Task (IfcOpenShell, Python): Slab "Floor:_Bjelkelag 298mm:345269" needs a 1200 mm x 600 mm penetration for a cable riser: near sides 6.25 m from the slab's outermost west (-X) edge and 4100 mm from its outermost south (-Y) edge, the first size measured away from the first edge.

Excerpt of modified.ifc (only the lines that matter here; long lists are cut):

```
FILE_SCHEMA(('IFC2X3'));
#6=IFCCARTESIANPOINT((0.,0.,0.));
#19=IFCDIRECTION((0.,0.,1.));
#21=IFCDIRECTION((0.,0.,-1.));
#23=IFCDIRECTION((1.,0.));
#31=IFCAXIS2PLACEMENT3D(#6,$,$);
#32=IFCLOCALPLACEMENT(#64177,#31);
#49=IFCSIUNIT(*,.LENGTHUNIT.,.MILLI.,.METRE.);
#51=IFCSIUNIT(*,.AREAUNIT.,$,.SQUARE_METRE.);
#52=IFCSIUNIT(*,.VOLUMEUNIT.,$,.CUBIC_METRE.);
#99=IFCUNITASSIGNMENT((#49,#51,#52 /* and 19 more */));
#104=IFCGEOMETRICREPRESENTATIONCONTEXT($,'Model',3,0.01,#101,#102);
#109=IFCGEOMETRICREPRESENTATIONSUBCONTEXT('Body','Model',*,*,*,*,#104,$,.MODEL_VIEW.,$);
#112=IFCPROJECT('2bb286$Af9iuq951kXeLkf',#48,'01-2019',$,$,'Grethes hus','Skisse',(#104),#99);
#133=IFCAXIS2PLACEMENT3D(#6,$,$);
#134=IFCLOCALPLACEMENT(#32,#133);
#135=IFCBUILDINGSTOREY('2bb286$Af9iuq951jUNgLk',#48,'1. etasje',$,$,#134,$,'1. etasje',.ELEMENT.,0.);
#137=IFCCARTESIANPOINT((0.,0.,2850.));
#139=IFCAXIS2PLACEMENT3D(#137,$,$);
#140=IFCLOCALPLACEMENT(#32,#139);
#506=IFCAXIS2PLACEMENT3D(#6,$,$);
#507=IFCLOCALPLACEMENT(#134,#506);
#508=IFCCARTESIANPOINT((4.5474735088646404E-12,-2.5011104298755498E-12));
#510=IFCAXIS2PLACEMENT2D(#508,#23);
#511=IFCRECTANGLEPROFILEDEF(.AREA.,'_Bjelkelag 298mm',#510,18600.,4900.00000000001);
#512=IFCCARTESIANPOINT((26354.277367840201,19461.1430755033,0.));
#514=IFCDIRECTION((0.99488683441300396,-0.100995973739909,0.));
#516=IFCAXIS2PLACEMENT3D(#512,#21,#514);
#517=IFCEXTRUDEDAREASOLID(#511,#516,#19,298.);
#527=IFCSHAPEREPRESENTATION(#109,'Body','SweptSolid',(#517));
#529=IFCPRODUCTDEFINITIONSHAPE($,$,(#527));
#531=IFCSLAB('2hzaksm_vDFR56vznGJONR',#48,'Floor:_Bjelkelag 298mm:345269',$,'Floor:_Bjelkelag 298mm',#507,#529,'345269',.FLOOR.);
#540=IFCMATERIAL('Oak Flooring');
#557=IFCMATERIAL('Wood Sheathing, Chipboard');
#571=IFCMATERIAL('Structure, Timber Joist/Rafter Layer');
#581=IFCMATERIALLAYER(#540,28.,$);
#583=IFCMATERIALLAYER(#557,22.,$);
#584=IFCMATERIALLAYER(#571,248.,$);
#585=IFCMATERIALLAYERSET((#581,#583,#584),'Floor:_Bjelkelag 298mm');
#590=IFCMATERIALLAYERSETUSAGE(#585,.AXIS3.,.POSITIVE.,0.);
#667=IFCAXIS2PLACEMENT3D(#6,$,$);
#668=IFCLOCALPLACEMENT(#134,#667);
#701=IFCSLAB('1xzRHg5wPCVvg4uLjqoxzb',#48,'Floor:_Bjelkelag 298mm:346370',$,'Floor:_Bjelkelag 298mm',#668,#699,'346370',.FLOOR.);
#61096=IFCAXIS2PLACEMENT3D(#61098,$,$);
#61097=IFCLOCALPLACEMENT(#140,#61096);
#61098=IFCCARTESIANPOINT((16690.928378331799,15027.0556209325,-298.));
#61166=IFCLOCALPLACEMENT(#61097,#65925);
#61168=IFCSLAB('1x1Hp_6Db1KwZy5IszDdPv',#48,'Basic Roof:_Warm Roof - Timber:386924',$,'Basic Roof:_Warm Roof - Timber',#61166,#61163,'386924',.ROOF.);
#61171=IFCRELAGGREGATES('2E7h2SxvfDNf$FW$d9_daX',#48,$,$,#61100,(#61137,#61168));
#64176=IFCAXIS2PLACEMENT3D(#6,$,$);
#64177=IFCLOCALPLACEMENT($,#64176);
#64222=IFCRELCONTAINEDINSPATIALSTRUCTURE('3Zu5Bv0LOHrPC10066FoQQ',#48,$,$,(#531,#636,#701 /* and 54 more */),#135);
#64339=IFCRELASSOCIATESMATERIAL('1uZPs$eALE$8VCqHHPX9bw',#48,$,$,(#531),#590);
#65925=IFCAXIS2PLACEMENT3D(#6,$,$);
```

```python
import numpy as np
import ifcopenshell
import ifcopenshell.api.feature
import ifcopenshell.api.geometry
import ifcopenshell.api.root
import ifcopenshell.geom
import ifcopenshell.util.placement
import ifcopenshell.util.representation
import ifcopenshell.util.shape
import ifcopenshell.util.unit

model = ifcopenshell.open("modified.ifc")
unit_scale = ifcopenshell.util.unit.calculate_unit_scale(model)
settings = ifcopenshell.geom.settings()


def volume(element):
    """Net volume in cubic metres, openings subtracted."""
    shape = ifcopenshell.geom.create_shape(settings, element)
    return ifcopenshell.util.shape.get_volume(shape.geometry)


slab = model.by_guid("2hzaksm_vDFR56vznGJONR")
before = volume(slab)

# Extent in the slab's own axes, in metres. The edges named are its -X and -Y sides.
slab_shape = ifcopenshell.geom.create_shape(settings, slab)
vertices = ifcopenshell.util.shape.get_vertices(slab_shape.geometry)
x_min, y_min, bottom = vertices.min(axis=0)
top = vertices[:, 2].max()

opening = ifcopenshell.api.root.create_entity(model, ifc_class="IfcOpeningElement", name="Cable riser opening")
context = ifcopenshell.util.representation.get_context(model, "Model", "Body", "MODEL_VIEW")
width, depth = 1.2, 0.6
outline = [(0.0, 0.0), (width, 0.0), (width, depth), (0.0, depth), (0.0, 0.0)]
# Overshoot both faces by 50 mm so the cut is clean.
shape = ifcopenshell.api.geometry.add_slab_representation(
    model, context=context, depth=top - bottom + 0.1, polyline=outline
)
ifcopenshell.api.geometry.assign_representation(model, product=opening, representation=shape)

matrix = ifcopenshell.util.placement.get_local_placement(slab.ObjectPlacement)
matrix[:, 3] = matrix @ np.append(np.array([x_min + 6.25, y_min + 4.1, bottom - 0.05]) / unit_scale, 1.0)
ifcopenshell.api.geometry.edit_object_placement(model, product=opening, matrix=matrix, is_si=False)
ifcopenshell.api.feature.add_feature(model, feature=opening, element=slab)

after = volume(slab)

print(f"slab volume {before:.3f} -> {after:.3f} m3")

model.write("modified_rev.ifc")
```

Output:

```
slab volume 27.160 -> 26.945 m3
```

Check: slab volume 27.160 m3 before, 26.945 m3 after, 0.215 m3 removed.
